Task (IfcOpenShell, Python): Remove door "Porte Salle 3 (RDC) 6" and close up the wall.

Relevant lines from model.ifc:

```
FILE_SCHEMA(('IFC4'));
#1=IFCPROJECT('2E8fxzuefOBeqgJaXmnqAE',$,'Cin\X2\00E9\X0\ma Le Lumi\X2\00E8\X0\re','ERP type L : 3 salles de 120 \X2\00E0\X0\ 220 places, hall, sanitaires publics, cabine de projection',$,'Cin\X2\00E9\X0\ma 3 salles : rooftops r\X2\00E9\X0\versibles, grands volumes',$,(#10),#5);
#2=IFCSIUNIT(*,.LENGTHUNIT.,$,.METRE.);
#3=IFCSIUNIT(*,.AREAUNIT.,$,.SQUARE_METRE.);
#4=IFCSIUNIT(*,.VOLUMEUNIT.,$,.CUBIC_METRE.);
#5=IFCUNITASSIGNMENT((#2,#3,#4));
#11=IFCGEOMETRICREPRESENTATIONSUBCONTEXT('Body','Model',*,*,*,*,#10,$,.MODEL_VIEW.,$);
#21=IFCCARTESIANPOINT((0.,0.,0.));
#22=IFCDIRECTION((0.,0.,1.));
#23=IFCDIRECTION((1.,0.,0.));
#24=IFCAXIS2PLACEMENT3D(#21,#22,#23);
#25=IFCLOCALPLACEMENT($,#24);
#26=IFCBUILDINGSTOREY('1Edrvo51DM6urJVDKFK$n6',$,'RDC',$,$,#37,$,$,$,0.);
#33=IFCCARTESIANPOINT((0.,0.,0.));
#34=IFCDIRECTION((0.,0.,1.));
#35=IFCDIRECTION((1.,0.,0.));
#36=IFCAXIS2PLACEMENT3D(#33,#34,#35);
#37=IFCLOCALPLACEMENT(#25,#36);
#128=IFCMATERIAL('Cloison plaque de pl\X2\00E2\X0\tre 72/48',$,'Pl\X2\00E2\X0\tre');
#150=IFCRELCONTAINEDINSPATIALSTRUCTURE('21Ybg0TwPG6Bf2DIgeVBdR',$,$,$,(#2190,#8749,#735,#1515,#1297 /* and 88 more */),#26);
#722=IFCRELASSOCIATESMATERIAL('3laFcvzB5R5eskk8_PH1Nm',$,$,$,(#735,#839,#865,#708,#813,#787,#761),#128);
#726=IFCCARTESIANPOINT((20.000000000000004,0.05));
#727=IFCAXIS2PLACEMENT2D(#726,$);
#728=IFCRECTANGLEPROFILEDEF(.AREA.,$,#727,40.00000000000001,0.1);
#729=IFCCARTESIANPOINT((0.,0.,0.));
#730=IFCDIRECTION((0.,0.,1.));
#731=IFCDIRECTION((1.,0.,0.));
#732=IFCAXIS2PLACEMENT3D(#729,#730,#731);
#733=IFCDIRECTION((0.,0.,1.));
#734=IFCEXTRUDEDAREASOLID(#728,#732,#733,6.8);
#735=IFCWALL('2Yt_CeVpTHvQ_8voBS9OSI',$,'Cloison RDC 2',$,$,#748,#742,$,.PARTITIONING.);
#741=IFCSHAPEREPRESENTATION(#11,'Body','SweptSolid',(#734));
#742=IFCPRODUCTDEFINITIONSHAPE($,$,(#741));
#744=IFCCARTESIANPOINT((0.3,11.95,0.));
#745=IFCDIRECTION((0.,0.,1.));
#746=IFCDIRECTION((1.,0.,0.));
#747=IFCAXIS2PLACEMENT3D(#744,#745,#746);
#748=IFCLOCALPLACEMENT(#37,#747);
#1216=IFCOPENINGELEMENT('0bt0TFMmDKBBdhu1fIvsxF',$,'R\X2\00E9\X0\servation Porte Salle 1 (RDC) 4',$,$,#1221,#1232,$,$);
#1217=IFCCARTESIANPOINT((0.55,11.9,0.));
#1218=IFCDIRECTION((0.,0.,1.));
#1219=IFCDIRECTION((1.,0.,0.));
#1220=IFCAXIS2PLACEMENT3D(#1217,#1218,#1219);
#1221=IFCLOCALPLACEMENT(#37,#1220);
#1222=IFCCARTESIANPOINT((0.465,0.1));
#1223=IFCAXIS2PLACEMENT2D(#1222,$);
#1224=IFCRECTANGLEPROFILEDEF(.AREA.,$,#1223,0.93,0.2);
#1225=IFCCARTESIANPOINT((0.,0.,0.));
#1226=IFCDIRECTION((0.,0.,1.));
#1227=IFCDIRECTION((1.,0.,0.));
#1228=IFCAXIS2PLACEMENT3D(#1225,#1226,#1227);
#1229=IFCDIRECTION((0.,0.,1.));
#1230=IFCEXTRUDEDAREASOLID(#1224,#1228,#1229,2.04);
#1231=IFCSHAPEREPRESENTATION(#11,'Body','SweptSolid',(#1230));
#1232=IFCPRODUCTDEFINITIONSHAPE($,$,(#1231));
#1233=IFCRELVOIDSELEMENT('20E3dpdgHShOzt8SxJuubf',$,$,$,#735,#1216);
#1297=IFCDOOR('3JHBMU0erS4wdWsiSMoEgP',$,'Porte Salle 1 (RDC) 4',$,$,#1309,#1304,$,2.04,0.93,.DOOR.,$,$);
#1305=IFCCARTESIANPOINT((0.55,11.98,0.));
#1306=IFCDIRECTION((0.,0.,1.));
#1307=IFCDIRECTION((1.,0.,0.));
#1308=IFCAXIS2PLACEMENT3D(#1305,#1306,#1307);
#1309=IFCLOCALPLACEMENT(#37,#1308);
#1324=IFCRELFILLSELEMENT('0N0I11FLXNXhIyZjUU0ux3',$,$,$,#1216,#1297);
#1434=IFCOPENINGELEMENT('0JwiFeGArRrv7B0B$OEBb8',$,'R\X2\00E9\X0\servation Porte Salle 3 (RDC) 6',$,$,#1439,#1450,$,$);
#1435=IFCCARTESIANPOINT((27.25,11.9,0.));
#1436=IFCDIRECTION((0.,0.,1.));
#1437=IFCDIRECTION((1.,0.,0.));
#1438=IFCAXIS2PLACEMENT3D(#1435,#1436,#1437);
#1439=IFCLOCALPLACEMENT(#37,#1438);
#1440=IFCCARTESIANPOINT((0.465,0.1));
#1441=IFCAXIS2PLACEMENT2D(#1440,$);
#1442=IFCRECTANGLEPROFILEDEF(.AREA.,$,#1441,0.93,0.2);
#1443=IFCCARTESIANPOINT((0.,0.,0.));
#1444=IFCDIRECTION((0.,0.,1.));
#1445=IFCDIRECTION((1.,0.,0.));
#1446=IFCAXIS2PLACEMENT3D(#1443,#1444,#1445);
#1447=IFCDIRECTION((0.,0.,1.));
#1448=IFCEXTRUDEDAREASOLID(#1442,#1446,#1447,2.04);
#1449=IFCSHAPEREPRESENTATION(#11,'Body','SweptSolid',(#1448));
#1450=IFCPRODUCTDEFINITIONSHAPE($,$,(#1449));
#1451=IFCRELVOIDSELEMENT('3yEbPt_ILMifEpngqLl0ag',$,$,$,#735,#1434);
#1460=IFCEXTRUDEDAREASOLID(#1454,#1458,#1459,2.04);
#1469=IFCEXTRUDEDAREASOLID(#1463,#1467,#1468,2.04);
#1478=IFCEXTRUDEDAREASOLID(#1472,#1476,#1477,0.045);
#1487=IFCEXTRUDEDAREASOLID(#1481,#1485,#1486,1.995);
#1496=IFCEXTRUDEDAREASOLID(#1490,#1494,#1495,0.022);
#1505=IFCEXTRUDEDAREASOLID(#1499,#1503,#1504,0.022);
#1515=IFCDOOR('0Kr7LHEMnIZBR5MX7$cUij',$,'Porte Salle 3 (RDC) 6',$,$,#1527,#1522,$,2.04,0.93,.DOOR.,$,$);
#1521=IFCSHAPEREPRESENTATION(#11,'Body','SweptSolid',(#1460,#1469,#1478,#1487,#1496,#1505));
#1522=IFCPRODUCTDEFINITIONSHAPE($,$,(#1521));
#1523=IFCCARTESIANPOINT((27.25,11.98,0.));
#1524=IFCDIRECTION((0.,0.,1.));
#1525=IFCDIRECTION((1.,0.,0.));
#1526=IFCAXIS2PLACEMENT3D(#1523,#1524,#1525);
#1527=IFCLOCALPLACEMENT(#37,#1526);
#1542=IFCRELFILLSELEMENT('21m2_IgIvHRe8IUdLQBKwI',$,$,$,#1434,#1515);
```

```python
import ifcopenshell
import ifcopenshell.api.feature
import ifcopenshell.api.root
import ifcopenshell.geom
import ifcopenshell.util.shape

model = ifcopenshell.open("model.ifc")
settings = ifcopenshell.geom.settings()


def volume(element):
    """Net volume in cubic metres, openings subtracted."""
    shape = ifcopenshell.geom.create_shape(settings, element)
    return ifcopenshell.util.shape.get_volume(shape.geometry)


door = model.by_guid("0Kr7LHEMnIZBR5MX7$cUij")
opening = door.FillsVoids[0].RelatingOpeningElement
wall = opening.VoidsElements[0].RelatingBuildingElement
before = volume(wall)

ifcopenshell.api.root.remove_product(model, product=door)
ifcopenshell.api.feature.remove_feature(model, feature=opening)

after = volume(wall)

print(f"wall volume {before:.3f} -> {after:.3f} m3")

model.write("model_edited.ifc")
```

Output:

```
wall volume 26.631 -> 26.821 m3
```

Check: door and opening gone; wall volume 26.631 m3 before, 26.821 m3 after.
